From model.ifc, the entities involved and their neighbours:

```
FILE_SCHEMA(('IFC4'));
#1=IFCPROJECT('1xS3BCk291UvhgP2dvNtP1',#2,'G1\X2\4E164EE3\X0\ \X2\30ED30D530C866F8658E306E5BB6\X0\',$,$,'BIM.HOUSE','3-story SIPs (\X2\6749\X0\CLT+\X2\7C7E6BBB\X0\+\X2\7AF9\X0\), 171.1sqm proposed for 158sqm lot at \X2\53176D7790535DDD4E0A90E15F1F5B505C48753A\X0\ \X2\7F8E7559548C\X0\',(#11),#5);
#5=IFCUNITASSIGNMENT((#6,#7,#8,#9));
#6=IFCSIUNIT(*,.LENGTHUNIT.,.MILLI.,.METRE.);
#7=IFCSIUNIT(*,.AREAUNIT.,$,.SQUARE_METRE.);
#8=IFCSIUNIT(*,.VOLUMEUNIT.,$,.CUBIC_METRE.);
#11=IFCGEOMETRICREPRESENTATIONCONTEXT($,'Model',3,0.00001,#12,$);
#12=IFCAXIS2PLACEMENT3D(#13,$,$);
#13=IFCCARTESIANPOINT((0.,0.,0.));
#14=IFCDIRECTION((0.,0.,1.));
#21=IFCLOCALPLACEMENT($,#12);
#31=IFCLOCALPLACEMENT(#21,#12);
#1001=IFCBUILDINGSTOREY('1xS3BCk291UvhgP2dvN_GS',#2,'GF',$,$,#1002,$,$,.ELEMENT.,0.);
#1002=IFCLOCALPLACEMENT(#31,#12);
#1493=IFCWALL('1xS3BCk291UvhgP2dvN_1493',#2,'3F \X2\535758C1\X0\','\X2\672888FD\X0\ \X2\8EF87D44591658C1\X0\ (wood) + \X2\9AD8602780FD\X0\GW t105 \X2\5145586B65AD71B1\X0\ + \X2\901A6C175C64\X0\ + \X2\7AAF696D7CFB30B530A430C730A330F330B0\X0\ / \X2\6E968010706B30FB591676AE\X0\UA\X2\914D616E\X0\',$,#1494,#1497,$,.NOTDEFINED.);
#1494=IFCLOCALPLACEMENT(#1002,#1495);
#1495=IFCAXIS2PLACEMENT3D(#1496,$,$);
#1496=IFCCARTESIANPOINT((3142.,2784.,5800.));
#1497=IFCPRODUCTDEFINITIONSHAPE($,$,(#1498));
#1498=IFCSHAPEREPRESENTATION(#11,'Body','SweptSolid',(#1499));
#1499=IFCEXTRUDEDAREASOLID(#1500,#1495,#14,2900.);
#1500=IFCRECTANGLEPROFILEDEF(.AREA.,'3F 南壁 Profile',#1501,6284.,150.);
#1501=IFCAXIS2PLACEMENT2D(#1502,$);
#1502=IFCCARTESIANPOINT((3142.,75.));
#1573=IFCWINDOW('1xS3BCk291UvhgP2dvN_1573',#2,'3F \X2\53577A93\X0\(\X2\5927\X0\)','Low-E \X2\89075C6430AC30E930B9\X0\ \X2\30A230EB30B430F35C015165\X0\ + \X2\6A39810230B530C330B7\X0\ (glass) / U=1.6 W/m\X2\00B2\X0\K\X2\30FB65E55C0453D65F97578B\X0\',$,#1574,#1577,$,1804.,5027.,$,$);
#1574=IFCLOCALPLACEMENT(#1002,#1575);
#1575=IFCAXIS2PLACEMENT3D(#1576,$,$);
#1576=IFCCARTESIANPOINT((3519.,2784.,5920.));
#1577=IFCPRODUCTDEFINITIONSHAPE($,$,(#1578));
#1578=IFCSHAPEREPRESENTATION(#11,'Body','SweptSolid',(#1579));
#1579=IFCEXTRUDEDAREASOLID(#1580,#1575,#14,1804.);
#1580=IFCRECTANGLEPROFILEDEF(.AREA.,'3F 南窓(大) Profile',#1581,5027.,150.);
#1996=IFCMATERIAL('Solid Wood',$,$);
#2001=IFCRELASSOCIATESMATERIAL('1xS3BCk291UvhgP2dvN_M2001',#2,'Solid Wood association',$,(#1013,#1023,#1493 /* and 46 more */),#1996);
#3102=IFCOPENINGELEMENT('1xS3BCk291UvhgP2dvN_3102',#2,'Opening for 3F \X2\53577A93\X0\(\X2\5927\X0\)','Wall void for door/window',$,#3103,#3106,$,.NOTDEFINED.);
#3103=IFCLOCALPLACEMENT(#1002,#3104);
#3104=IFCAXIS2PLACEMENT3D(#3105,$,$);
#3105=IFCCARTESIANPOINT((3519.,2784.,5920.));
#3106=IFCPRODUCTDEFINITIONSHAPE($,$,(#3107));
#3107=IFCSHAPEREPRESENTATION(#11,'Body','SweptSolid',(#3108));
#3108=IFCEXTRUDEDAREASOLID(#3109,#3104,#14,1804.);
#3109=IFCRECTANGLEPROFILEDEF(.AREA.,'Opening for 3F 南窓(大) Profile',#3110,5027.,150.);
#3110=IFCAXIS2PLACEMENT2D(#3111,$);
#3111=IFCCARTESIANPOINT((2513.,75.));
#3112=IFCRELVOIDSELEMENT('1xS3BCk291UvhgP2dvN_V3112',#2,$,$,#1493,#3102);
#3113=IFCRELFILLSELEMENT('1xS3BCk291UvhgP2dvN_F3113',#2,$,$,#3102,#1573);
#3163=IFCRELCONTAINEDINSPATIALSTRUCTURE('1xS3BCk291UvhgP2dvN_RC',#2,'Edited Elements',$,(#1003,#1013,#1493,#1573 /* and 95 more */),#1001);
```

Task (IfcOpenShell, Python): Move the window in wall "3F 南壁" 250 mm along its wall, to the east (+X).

```python
import ifcopenshell
import ifcopenshell.api.geometry
import ifcopenshell.util.placement

model = ifcopenshell.open("model.ifc")

window = model.by_guid("1xS3BCk291UvhgP2dvN_1573")
opening = window.FillsVoids[0].RelatingOpeningElement
wall = opening.VoidsElements[0].RelatingBuildingElement

wall_matrix = ifcopenshell.util.placement.get_local_placement(wall.ObjectPlacement)
shift = wall_matrix[:3, 0] * 250.0
before = ifcopenshell.util.placement.get_local_placement(window.ObjectPlacement)[:3, 3].copy()

# The window is not placed relative to its opening, so move both.
for product in (opening, window):
    matrix = ifcopenshell.util.placement.get_local_placement(product.ObjectPlacement)
    matrix[:3, 3] += shift
    ifcopenshell.api.geometry.edit_object_placement(model, product=product, matrix=matrix, is_si=False)

after = ifcopenshell.util.placement.get_local_placement(window.ObjectPlacement)[:3, 3]
print("window moved by", (after - before).round(3) + 0.0)

model.write("model_v2.ifc")
```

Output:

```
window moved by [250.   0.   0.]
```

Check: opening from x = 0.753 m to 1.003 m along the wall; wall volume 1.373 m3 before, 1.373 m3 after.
